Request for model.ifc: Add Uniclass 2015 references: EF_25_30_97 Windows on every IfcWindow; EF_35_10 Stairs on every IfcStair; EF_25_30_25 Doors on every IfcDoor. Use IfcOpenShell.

First a look at what the model holds.

```python
import ifcopenshell

model = ifcopenshell.open("model.ifc")
print(model.schema)
print("classifications:", [c.Name for c in model.by_type("IfcClassification")])
for ifc_class in ("IfcDoor", "IfcRoof", "IfcStair", "IfcWall", "IfcWindow"):
    print(ifc_class, len(model.by_type(ifc_class)))
```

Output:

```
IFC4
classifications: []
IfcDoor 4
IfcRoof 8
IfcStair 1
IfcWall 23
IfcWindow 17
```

```python
import ifcopenshell
import ifcopenshell.api.classification

model = ifcopenshell.open("model.ifc")

system = ifcopenshell.api.classification.add_classification(model, classification="Uniclass 2015")

codes = {
    "IfcWindow": ("EF_25_30_97", "Windows"),
    "IfcStair": ("EF_35_10", "Stairs"),
    "IfcDoor": ("EF_25_30_25", "Doors"),
}
for ifc_class, (code, name) in codes.items():
    products = model.by_type(ifc_class)
    ifcopenshell.api.classification.add_reference(
        model, products=products, classification=system, identification=code, name=name
    )
    print(code, len(products))

model.write("model_rev.ifc")
```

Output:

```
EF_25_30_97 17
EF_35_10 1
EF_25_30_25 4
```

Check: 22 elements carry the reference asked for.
